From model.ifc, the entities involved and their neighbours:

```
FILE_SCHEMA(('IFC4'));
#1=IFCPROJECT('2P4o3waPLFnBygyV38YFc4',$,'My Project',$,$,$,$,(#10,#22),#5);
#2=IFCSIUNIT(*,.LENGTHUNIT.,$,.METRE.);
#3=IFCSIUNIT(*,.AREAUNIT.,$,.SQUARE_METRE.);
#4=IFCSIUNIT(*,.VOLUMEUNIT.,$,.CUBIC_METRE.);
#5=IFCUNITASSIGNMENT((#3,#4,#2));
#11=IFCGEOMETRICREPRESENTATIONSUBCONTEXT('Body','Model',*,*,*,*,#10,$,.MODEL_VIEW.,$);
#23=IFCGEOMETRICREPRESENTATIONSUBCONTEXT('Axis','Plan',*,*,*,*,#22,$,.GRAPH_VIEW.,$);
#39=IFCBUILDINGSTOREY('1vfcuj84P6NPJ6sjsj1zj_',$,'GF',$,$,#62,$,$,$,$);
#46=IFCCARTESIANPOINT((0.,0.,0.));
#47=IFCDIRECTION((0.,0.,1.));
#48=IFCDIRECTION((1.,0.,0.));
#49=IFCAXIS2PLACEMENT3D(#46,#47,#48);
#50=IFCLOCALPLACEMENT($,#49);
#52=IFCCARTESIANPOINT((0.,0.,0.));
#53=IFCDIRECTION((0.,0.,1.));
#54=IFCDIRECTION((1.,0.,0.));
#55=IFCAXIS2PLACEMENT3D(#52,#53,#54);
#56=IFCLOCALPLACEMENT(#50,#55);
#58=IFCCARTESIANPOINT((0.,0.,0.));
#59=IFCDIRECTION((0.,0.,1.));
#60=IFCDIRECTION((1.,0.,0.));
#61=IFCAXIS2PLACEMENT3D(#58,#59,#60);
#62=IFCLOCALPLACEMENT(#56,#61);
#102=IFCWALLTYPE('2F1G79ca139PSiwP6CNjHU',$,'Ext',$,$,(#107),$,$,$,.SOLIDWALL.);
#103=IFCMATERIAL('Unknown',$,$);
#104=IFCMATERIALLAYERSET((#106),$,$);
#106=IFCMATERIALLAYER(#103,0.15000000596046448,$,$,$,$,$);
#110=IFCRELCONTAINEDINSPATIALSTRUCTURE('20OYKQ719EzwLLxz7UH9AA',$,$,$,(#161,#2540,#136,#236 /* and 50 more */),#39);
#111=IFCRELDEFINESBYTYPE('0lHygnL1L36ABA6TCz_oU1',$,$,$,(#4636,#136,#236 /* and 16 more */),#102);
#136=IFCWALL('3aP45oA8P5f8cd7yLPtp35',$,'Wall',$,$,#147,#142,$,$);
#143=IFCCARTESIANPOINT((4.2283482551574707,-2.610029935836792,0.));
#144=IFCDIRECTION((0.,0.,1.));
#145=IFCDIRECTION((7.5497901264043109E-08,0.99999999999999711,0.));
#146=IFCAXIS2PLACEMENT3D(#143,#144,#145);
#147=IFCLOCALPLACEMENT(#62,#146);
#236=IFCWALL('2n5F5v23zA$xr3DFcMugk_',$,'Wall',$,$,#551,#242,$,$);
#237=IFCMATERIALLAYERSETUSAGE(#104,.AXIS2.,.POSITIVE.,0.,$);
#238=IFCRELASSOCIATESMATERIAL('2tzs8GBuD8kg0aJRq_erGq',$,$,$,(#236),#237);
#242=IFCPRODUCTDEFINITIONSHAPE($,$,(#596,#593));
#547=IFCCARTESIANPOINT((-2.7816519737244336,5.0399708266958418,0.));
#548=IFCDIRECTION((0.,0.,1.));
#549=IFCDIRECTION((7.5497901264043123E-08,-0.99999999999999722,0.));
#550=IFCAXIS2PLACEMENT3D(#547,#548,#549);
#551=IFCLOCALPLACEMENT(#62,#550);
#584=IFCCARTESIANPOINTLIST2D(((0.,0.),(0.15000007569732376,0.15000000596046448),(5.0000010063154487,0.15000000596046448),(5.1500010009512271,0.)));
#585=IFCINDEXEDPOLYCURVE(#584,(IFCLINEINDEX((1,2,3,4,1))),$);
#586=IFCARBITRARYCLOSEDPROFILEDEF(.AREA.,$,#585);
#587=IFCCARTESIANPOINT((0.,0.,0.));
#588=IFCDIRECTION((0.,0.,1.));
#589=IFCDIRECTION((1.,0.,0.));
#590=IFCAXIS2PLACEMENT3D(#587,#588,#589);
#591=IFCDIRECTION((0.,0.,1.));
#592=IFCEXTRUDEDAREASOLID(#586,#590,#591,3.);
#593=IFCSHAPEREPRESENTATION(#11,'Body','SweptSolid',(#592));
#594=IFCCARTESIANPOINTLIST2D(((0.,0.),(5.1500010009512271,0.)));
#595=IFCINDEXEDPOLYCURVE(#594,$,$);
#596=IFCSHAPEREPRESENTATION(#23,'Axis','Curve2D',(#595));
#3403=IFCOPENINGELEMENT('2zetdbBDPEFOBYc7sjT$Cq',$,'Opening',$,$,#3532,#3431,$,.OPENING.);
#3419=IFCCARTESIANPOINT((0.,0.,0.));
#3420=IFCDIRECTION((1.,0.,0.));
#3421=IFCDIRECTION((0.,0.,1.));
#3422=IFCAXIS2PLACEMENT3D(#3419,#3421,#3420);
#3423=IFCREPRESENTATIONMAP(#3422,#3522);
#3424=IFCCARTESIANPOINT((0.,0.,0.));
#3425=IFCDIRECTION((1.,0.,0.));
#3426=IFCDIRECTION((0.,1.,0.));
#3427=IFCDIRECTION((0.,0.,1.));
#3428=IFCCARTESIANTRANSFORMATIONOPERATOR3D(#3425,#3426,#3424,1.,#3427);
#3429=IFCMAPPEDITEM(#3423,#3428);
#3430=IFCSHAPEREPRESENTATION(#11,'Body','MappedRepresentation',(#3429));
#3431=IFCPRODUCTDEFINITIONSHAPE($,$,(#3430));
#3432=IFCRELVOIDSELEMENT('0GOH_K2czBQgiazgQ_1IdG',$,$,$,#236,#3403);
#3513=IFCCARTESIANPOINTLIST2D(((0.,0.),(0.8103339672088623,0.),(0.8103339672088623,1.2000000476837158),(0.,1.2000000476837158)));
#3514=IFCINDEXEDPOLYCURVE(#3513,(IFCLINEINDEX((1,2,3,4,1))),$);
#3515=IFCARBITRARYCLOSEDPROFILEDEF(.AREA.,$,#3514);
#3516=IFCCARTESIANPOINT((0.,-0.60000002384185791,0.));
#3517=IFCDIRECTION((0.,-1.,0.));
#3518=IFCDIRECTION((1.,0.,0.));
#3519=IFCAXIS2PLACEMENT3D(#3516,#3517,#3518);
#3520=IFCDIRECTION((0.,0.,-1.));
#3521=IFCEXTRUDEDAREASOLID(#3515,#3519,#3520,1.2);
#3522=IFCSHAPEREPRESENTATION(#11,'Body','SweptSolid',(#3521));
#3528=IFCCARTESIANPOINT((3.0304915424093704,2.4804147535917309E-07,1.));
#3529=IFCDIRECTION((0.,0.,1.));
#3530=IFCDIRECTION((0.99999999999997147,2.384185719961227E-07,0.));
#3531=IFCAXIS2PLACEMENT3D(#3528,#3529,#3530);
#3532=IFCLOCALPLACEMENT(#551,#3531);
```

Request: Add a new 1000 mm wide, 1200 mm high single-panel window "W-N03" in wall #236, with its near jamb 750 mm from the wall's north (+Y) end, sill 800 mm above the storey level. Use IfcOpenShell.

```python
import numpy as np
import ifcopenshell
import ifcopenshell.api.feature
import ifcopenshell.api.geometry
import ifcopenshell.api.root
import ifcopenshell.api.spatial
import ifcopenshell.geom
import ifcopenshell.util.element
import ifcopenshell.util.placement
import ifcopenshell.util.representation
import ifcopenshell.util.shape
import ifcopenshell.util.unit

model = ifcopenshell.open("model.ifc")
unit_scale = ifcopenshell.util.unit.calculate_unit_scale(model)
settings = ifcopenshell.geom.settings()


def volume(element):
    """Net volume in cubic metres, openings subtracted."""
    shape = ifcopenshell.geom.create_shape(settings, element)
    return ifcopenshell.util.shape.get_volume(shape.geometry)


wall = model.by_id(236)
storey = ifcopenshell.util.element.get_container(wall, ifc_class="IfcBuildingStorey")
context = ifcopenshell.util.representation.get_context(model, "Model", "Body", "MODEL_VIEW")
before = volume(wall)

width, height, from_end, sill = 1, 1.2, 0.75, 0.8  # metres

# The wall runs along its own X axis, and the end named is its -X end.
wall_shape = ifcopenshell.geom.create_shape(settings, wall)
x, y, z = ifcopenshell.util.shape.get_vertices(wall_shape.geometry).T
start = x.min() + from_end
face, thickness = float(y.min()), float(y.max() - y.min())
wall_matrix = ifcopenshell.util.placement.get_local_placement(wall.ObjectPlacement)
level = ifcopenshell.util.placement.get_local_placement(storey.ObjectPlacement)[2, 3]


def in_wall(x, y):
    """Placement at x, y metres in the wall's axes, at sill height."""
    matrix = wall_matrix.copy()
    matrix[:, 3] = wall_matrix @ np.array([x / unit_scale, y / unit_scale, 0.0, 1.0])
    matrix[2, 3] = level + sill / unit_scale
    return matrix


# Opening: a box that overshoots both wall faces by 50 mm.
opening = ifcopenshell.api.root.create_entity(model, ifc_class="IfcOpeningElement", predefined_type="OPENING")
box = ifcopenshell.api.geometry.add_wall_representation(
    model, context=context, length=width, height=height, thickness=thickness + 0.1
)
ifcopenshell.api.geometry.assign_representation(model, product=opening, representation=box)
ifcopenshell.api.geometry.edit_object_placement(model, product=opening, matrix=in_wall(start, face - 0.05), is_si=False)
ifcopenshell.api.feature.add_feature(model, feature=opening, element=wall)

window = ifcopenshell.api.root.create_entity(model, ifc_class="IfcWindow", name="W-N03", predefined_type="WINDOW")
window.OverallWidth, window.OverallHeight = width / unit_scale, height / unit_scale
window.PartitioningType = "SINGLE_PANEL"
body = ifcopenshell.api.geometry.add_window_representation(
    model,
    context=context,
    overall_width=window.OverallWidth,
    overall_height=window.OverallHeight,
    partition_type="SINGLE_PANEL",
)
ifcopenshell.api.geometry.assign_representation(model, product=window, representation=body)
ifcopenshell.api.spatial.assign_container(model, products=[window], relating_structure=storey)
ifcopenshell.api.feature.add_filling(model, opening=opening, element=window)

# Centre the window in the wall's thickness.
ifcopenshell.api.geometry.edit_object_placement(model, product=window, matrix=in_wall(start, face), is_si=False)
window_shape = ifcopenshell.geom.create_shape(settings, window)
depth = ifcopenshell.util.shape.get_vertices(window_shape.geometry)[:, 1]
offset = face + thickness / 2 - (depth.min() + depth.max()) / 2
ifcopenshell.api.geometry.edit_object_placement(model, product=window, matrix=in_wall(start, offset), is_si=False)

after = volume(wall)

print(f"wall volume {before:.3f} -> {after:.3f} m3")

model.write("model_updated.ifc")
```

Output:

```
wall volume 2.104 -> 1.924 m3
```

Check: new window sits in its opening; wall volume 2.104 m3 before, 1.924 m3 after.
